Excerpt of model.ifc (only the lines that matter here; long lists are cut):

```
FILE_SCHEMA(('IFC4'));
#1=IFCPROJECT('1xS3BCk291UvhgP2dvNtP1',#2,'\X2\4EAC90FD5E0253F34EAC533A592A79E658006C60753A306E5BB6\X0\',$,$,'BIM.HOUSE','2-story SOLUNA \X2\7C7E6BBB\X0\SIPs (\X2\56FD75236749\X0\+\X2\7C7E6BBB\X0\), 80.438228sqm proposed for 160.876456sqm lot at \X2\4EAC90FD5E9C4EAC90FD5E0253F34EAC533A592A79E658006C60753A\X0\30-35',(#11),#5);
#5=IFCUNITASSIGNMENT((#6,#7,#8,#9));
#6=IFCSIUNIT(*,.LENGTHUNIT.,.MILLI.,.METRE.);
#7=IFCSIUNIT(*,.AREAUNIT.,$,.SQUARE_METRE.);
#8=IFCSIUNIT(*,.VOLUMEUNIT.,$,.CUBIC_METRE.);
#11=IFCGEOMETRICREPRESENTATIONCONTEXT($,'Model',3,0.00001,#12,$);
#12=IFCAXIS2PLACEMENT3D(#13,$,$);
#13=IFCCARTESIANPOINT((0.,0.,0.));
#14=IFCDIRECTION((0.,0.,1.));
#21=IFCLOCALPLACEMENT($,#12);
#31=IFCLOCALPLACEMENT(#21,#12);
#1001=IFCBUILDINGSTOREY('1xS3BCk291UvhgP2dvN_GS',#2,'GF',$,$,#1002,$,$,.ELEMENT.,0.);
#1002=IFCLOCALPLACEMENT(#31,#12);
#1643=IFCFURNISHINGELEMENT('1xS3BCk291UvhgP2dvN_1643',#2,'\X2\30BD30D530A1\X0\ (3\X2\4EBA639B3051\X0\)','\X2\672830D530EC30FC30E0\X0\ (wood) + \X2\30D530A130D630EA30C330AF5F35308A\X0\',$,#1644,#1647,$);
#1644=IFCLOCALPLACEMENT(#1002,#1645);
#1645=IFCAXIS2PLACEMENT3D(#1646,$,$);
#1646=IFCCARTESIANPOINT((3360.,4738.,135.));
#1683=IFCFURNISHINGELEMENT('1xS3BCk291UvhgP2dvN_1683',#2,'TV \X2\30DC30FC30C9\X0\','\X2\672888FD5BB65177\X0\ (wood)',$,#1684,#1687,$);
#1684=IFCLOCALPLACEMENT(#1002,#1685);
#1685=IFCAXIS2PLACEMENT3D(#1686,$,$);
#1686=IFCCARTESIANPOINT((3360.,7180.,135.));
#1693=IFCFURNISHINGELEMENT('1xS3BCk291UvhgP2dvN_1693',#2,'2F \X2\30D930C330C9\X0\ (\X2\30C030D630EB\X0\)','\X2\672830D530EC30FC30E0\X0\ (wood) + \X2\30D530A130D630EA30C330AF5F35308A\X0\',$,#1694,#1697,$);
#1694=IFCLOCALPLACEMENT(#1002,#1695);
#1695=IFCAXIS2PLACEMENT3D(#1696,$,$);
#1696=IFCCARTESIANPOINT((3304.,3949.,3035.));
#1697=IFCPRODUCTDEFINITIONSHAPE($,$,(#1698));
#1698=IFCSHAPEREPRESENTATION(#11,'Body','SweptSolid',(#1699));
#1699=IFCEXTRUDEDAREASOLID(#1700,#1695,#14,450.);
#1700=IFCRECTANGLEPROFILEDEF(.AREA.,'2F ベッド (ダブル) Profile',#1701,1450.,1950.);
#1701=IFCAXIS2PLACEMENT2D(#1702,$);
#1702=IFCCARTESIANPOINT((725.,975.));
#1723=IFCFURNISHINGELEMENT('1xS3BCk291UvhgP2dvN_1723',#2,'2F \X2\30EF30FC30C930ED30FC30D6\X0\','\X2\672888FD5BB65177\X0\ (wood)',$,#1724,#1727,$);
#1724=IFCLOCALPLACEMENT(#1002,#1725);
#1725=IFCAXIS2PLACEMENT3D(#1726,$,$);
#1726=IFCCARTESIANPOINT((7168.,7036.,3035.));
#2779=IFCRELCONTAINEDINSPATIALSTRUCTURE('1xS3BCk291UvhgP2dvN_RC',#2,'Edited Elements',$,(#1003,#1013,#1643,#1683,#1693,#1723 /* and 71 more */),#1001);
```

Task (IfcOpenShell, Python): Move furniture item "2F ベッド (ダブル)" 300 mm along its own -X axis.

```python
import ifcopenshell
import ifcopenshell.api.geometry
import ifcopenshell.util.placement

model = ifcopenshell.open("model.ifc")

item = model.by_guid("1xS3BCk291UvhgP2dvN_1693")
matrix = ifcopenshell.util.placement.get_local_placement(item.ObjectPlacement)
matrix[:3, 3] -= matrix[:3, 0] * 300.0
ifcopenshell.api.geometry.edit_object_placement(model, product=item, matrix=matrix, is_si=False)

print(ifcopenshell.util.placement.get_local_placement(item.ObjectPlacement).round(3) + 0.0)

model.write("model-out.ifc")
```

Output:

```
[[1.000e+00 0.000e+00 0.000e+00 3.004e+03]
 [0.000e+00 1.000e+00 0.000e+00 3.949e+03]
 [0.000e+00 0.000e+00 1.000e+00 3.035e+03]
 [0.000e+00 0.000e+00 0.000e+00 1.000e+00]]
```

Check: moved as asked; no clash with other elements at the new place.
